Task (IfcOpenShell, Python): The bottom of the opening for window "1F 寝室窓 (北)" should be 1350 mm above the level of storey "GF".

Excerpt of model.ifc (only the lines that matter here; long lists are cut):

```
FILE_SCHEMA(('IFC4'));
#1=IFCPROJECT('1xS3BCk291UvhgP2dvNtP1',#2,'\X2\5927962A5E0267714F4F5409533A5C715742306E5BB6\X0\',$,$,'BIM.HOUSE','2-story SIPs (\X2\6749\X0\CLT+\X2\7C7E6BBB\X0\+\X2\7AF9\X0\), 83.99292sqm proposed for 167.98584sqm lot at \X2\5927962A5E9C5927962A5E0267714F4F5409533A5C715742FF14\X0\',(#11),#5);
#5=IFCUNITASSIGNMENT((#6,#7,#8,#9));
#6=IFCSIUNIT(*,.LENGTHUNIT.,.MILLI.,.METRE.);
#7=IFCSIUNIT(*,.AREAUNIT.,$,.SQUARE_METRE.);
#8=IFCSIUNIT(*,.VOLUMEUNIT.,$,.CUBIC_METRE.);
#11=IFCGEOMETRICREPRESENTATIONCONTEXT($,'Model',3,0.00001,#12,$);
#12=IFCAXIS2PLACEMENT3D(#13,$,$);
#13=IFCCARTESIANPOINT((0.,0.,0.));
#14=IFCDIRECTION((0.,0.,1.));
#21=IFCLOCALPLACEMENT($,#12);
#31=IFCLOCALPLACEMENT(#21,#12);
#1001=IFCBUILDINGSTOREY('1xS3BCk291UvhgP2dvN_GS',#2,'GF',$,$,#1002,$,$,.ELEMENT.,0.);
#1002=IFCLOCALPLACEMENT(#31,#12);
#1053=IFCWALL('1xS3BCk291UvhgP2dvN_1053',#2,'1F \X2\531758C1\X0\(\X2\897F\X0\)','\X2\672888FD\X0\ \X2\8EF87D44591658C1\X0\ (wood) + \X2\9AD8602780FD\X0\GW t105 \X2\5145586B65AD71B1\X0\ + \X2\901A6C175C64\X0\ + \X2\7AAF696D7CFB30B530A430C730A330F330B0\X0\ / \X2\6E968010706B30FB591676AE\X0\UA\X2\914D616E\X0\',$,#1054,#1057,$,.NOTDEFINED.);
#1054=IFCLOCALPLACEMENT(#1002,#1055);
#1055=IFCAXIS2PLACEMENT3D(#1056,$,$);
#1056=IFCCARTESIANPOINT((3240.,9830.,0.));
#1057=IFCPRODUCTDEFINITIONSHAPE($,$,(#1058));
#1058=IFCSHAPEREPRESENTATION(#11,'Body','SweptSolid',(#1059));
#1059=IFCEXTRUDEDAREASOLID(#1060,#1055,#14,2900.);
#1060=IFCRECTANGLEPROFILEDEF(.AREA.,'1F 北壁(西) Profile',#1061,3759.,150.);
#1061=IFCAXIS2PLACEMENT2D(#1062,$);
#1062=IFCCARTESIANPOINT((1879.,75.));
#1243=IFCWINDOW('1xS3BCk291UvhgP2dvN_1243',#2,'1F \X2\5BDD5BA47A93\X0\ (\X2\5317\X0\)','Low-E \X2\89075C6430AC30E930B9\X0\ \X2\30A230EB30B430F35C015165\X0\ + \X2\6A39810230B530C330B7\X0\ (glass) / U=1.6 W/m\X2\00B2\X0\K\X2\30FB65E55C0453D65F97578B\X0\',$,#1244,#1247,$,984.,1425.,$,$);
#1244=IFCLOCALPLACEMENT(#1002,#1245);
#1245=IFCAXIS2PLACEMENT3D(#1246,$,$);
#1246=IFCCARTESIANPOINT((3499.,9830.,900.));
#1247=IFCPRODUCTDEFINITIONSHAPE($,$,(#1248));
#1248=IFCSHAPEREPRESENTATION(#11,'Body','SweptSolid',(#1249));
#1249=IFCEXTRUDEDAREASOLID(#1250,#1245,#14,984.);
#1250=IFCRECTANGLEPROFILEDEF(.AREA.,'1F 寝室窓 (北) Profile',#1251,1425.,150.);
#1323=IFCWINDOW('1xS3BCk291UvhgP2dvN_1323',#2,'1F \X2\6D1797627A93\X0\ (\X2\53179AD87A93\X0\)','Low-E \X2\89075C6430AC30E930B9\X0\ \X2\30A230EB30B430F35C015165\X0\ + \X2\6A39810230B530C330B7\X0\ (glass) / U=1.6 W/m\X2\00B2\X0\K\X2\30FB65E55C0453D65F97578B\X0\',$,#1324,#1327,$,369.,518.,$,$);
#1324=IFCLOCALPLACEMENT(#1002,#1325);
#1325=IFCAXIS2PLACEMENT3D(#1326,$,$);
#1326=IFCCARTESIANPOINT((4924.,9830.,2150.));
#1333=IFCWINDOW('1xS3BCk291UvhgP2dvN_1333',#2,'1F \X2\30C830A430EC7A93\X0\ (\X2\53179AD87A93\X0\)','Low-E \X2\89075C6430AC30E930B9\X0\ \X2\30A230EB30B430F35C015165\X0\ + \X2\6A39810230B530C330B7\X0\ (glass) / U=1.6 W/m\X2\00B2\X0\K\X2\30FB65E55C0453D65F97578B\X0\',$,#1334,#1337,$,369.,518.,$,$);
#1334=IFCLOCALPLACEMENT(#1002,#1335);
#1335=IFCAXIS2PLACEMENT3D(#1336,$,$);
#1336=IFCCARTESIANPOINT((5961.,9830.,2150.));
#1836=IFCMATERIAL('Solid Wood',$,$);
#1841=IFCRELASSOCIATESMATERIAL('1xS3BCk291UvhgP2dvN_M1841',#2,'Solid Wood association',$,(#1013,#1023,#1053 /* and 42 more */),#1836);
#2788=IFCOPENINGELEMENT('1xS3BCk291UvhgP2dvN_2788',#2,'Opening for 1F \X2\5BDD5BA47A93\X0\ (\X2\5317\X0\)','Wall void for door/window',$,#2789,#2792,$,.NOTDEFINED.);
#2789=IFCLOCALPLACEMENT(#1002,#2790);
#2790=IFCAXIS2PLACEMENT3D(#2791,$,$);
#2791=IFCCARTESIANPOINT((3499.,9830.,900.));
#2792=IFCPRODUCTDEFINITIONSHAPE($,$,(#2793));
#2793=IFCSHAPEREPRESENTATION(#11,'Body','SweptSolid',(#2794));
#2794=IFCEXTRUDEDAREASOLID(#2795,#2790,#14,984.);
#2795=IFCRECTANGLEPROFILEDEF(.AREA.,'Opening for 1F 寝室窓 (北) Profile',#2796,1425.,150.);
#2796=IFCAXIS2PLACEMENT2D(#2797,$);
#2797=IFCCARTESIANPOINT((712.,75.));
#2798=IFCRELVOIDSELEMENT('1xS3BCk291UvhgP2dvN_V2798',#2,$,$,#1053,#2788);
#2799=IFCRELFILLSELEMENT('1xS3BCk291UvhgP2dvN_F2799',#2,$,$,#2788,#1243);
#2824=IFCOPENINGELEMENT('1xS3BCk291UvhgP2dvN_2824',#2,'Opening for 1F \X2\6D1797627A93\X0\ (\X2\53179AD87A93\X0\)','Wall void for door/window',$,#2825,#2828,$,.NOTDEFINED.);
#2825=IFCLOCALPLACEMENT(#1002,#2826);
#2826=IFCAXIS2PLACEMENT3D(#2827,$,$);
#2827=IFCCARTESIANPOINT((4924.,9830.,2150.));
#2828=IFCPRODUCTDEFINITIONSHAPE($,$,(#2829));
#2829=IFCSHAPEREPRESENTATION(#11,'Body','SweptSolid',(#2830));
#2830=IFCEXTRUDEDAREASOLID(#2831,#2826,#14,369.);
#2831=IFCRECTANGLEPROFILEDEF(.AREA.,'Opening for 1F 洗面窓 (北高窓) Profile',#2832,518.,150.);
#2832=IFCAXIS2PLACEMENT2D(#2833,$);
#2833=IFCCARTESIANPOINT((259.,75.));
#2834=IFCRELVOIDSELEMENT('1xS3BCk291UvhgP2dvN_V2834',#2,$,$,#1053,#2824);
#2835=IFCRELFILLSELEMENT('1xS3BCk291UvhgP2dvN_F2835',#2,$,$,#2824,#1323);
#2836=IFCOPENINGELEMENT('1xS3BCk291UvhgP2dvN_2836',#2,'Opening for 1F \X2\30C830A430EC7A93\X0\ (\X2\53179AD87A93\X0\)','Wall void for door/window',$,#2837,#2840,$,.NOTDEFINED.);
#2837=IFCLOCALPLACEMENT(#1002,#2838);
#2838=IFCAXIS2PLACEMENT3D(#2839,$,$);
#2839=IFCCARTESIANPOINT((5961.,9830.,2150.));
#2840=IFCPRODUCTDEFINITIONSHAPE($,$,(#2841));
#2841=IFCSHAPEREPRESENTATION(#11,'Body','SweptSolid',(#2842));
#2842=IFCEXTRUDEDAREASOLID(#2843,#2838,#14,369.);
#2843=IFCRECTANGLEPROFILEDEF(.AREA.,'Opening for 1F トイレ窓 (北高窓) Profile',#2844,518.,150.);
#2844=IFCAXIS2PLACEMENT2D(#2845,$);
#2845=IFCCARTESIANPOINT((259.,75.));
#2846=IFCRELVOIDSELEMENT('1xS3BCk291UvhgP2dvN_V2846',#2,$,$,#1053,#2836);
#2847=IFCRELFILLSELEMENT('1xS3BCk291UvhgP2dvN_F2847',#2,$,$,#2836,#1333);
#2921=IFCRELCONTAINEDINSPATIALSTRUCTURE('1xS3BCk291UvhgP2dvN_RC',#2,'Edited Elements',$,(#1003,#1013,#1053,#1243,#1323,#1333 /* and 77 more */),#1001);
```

```python
import numpy as np
import ifcopenshell
import ifcopenshell.api.geometry
import ifcopenshell.geom
import ifcopenshell.util.element
import ifcopenshell.util.placement
import ifcopenshell.util.shape
import ifcopenshell.util.unit

model = ifcopenshell.open("model.ifc")
unit_scale = ifcopenshell.util.unit.calculate_unit_scale(model)

window = model.by_id(1243)
opening = window.FillsVoids[0].RelatingOpeningElement
storey = ifcopenshell.util.element.get_container(window, ifc_class="IfcBuildingStorey")
level = ifcopenshell.util.placement.get_local_placement(storey.ObjectPlacement)[2, 3]

# The opening's origin need not be at the sill, so measure its lowest point.
shape = ifcopenshell.geom.create_shape(ifcopenshell.geom.settings(), opening)
bottom = ifcopenshell.util.shape.get_shape_bottom_elevation(shape, shape.geometry) / unit_scale
dz = level + 1.35 / unit_scale - bottom

shift = np.array([0.0, 0.0, dz])
# The window is not placed relative to its opening, so move both.
for product in (opening, window):
    matrix = ifcopenshell.util.placement.get_local_placement(product.ObjectPlacement)
    matrix[:3, 3] += shift
    ifcopenshell.api.geometry.edit_object_placement(model, product=product, matrix=matrix, is_si=False)

print(f"moved by {dz * unit_scale:+.3f} m")

model.write("model_edited.ifc")
```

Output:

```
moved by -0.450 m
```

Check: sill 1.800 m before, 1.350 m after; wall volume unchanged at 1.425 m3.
